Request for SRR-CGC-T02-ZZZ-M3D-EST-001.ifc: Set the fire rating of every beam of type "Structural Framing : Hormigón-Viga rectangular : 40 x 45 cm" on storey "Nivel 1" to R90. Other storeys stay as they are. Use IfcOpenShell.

First a look at what the model holds.

```python
import ifcopenshell
import ifcopenshell.util.element

model = ifcopenshell.open("SRR-CGC-T02-ZZZ-M3D-EST-001.ifc")
print(model.schema)
storey = next(s for s in model.by_type("IfcBuildingStorey") if s.Name == "Nivel 1")
beams = [e for e in ifcopenshell.util.element.get_decomposition(storey) if e.is_a("IfcBeam")]
seen = {}
for e in beams:
    element_type = ifcopenshell.util.element.get_type(e)
    key = (element_type.Name if element_type != e and element_type else None, ifcopenshell.util.element.get_pset(e, "Pset_BeamCommon", "FireRating"))
    seen[key] = seen.get(key, 0) + 1
for (name, value), count in sorted(seen.items(), key=str):
    print(count, "x", name, "|", value)
```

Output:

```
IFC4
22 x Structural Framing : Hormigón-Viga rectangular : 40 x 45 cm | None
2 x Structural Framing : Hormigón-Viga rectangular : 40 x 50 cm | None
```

```python
import ifcopenshell
import ifcopenshell.api.pset
import ifcopenshell.util.element

model = ifcopenshell.open("SRR-CGC-T02-ZZZ-M3D-EST-001.ifc")

storey = next(s for s in model.by_type("IfcBuildingStorey") if s.Name == "Nivel 1")
beams = [e for e in ifcopenshell.util.element.get_decomposition(storey) if e.is_a("IfcBeam")]

count = 0
for e in beams:
    element_type = ifcopenshell.util.element.get_type(e)
    if element_type in (None, e) or element_type.Name != "Structural Framing : Hormigón-Viga rectangular : 40 x 45 cm":
        continue
    # add_pset returns the element's existing set when there is one.
    pset = ifcopenshell.api.pset.add_pset(model, product=e, name="Pset_BeamCommon")
    ifcopenshell.api.pset.edit_pset(model, pset=pset, properties={"FireRating": "R90"})
    count += 1

print(count, "beams updated")

model.write("SRR-CGC-T02-ZZZ-M3D-EST-001-out.ifc")
```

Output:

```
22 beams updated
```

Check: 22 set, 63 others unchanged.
